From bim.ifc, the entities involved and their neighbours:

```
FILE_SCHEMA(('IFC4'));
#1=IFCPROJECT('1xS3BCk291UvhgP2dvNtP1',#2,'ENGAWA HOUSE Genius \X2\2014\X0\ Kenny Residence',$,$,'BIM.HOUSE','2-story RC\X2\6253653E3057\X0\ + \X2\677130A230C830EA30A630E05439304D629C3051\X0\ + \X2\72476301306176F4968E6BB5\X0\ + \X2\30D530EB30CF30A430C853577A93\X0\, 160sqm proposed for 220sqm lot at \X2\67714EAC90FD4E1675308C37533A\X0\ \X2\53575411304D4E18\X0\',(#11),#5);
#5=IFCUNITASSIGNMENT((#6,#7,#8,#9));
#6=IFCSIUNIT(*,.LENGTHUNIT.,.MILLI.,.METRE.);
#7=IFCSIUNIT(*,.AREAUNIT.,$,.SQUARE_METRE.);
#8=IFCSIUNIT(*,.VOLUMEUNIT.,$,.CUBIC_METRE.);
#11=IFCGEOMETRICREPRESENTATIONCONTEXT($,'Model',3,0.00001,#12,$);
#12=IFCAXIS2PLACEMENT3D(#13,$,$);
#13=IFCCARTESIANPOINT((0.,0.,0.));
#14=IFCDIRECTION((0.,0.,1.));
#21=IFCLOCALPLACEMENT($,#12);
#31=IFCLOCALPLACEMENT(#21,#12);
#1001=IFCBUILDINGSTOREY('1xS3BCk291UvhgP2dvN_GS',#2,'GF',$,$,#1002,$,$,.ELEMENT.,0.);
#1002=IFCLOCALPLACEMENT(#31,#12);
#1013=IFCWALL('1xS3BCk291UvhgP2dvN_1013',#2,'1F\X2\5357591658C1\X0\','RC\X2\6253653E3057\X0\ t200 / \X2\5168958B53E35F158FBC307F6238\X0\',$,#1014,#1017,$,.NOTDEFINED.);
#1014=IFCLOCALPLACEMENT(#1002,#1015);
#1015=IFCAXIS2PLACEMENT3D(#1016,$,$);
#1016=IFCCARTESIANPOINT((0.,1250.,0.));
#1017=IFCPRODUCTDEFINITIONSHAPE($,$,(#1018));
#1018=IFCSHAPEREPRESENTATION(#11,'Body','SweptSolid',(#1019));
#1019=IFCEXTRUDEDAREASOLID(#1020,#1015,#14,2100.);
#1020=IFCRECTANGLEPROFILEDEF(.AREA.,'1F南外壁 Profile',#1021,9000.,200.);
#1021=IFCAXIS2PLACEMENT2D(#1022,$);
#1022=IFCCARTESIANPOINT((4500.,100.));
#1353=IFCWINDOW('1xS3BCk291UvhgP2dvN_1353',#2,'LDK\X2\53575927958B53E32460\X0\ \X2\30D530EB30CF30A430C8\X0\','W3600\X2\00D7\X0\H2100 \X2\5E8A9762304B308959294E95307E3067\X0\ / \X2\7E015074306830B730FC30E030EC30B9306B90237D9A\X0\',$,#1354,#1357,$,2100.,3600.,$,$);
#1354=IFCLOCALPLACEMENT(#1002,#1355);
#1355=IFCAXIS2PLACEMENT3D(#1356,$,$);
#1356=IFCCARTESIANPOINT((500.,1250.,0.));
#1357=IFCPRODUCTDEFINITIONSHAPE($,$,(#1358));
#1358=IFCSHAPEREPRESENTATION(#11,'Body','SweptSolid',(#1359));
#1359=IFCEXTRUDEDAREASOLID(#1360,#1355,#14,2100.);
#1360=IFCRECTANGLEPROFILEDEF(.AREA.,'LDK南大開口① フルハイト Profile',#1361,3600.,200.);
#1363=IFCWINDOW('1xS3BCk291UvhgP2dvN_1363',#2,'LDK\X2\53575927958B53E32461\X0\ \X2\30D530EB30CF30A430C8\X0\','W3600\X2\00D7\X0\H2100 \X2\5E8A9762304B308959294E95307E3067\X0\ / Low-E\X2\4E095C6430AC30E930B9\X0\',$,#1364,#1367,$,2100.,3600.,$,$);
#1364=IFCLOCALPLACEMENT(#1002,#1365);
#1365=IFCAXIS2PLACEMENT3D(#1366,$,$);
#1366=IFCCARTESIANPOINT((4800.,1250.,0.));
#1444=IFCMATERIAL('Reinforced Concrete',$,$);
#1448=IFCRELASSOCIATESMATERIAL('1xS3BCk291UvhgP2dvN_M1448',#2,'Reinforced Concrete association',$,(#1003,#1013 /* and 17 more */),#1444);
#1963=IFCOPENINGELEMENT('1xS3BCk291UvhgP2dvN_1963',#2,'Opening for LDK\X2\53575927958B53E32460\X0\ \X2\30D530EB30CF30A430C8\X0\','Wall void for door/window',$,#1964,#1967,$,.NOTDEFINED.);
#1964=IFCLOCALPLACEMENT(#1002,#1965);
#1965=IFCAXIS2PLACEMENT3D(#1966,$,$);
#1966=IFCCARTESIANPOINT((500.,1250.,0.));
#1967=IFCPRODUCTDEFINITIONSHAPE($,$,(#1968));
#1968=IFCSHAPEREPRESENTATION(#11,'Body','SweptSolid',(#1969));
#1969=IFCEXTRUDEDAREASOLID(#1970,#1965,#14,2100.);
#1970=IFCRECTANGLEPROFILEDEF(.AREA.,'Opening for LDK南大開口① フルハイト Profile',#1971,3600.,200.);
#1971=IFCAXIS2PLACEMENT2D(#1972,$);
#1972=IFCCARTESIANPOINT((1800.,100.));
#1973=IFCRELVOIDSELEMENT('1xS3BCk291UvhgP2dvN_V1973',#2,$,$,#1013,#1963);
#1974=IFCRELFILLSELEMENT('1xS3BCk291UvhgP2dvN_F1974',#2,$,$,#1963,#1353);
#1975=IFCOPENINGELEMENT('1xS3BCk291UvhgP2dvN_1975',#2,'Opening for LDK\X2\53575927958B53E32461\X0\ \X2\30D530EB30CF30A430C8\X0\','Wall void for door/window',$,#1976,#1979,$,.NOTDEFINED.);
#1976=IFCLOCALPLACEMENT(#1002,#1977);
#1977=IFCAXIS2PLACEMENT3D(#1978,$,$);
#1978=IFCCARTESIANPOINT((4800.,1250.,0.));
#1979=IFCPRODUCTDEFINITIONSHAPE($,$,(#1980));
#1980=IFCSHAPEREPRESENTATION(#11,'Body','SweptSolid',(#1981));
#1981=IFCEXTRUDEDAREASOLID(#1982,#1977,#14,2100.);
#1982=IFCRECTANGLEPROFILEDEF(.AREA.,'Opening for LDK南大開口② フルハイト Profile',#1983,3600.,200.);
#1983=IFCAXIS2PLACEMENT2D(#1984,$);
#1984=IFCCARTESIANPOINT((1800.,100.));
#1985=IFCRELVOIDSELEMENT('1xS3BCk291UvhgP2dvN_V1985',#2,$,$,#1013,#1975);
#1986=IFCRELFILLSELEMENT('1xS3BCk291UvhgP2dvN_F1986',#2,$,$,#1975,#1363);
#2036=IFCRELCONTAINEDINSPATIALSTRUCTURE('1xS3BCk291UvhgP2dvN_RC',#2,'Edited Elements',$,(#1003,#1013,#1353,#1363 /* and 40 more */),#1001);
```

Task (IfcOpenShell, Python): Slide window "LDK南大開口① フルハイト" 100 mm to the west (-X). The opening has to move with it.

```python
import ifcopenshell
import ifcopenshell.api.geometry
import ifcopenshell.util.placement
import ifcopenshell.util.unit

model = ifcopenshell.open("bim.ifc")
unit_scale = ifcopenshell.util.unit.calculate_unit_scale(model)

window = model.by_guid("1xS3BCk291UvhgP2dvN_1353")
opening = window.FillsVoids[0].RelatingOpeningElement
wall = opening.VoidsElements[0].RelatingBuildingElement

wall_matrix = ifcopenshell.util.placement.get_local_placement(wall.ObjectPlacement)
shift = wall_matrix[:3, 0] * -0.1 / unit_scale
before = ifcopenshell.util.placement.get_local_placement(window.ObjectPlacement)[:3, 3].copy()

# The window is not placed relative to its opening, so move both.
for product in (opening, window):
    matrix = ifcopenshell.util.placement.get_local_placement(product.ObjectPlacement)
    matrix[:3, 3] += shift
    ifcopenshell.api.geometry.edit_object_placement(model, product=product, matrix=matrix, is_si=False)

after = ifcopenshell.util.placement.get_local_placement(window.ObjectPlacement)[:3, 3]
print("window moved by", (after - before).round(3) + 0.0)

model.write("bim-out.ifc")
```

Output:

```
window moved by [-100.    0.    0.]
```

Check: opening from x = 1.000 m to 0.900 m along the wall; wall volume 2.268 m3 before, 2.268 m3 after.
